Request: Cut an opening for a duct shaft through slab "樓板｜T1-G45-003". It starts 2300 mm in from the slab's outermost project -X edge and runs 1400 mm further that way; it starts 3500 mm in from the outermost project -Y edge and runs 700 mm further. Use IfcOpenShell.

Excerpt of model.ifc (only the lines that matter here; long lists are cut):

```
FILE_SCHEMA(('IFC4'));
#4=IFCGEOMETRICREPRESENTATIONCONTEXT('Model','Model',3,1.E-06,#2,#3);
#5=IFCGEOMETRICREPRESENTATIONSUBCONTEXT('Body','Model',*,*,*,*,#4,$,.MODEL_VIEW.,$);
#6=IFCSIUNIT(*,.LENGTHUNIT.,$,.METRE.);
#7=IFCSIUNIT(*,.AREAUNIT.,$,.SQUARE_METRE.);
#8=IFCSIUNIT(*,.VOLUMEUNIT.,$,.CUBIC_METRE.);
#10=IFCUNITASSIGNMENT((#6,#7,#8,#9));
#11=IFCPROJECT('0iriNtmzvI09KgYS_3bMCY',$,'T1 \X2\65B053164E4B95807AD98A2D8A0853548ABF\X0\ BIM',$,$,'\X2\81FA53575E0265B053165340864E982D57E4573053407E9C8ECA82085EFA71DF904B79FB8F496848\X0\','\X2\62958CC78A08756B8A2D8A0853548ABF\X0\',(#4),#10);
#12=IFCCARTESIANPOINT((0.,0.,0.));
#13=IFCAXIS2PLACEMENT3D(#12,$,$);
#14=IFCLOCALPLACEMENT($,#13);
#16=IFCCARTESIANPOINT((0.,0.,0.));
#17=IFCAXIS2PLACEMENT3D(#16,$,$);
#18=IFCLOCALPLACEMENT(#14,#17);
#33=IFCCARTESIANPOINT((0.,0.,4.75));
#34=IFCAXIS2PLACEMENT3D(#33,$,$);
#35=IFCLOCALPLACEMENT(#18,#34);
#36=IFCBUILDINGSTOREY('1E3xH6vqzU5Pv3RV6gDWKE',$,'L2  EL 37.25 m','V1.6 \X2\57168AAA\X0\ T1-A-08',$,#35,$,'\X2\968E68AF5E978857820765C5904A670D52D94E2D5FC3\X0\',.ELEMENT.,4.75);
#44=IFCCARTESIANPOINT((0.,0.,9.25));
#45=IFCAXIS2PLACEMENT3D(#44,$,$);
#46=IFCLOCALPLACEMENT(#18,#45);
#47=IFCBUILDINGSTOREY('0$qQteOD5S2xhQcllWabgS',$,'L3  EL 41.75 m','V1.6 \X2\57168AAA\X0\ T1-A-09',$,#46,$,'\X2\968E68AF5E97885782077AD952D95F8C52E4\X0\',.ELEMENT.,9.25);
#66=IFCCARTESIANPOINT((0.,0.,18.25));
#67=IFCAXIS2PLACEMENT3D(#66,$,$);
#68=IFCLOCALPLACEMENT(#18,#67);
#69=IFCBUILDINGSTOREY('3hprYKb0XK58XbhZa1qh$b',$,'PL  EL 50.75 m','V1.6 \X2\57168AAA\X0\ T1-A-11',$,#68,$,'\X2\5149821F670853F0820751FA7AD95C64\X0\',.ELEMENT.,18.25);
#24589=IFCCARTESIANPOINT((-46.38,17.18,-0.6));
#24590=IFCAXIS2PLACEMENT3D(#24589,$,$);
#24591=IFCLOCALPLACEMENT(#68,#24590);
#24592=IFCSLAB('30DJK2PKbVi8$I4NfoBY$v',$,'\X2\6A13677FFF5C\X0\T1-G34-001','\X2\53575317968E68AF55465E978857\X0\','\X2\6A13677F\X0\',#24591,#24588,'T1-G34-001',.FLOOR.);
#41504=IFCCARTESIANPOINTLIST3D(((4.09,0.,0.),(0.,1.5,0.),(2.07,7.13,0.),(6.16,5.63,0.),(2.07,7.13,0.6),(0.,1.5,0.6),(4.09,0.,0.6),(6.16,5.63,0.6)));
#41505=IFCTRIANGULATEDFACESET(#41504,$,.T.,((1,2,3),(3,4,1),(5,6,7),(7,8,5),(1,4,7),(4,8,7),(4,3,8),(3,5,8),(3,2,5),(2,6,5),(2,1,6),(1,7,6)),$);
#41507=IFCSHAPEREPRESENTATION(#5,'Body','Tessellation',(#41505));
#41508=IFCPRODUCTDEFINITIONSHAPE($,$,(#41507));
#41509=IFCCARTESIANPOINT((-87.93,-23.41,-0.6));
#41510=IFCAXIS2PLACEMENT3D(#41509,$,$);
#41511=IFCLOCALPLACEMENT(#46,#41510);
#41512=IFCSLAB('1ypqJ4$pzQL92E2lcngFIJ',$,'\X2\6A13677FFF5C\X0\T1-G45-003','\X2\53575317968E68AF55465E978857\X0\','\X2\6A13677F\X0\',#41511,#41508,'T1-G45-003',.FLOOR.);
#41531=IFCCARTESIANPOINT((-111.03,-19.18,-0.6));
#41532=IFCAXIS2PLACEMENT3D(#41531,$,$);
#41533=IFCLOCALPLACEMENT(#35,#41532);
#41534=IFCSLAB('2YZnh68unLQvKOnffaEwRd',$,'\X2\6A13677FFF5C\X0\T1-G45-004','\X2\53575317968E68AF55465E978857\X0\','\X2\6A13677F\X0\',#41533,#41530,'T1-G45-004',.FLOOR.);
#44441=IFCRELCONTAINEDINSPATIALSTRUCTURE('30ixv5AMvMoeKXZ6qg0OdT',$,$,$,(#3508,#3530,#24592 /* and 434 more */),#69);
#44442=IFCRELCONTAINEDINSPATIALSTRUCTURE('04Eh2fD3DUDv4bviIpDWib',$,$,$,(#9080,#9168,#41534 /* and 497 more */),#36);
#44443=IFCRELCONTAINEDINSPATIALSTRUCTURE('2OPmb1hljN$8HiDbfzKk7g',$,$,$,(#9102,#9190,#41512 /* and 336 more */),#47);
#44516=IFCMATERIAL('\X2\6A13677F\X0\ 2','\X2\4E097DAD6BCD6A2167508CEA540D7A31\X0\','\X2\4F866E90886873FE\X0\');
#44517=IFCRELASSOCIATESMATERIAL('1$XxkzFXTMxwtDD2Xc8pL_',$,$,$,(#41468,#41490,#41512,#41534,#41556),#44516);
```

```python
import numpy as np
import ifcopenshell
import ifcopenshell.api.feature
import ifcopenshell.api.geometry
import ifcopenshell.api.root
import ifcopenshell.geom
import ifcopenshell.util.placement
import ifcopenshell.util.representation
import ifcopenshell.util.shape
import ifcopenshell.util.unit

model = ifcopenshell.open("model.ifc")
unit_scale = ifcopenshell.util.unit.calculate_unit_scale(model)
settings = ifcopenshell.geom.settings()


def volume(element):
    """Net volume in cubic metres, openings subtracted."""
    shape = ifcopenshell.geom.create_shape(settings, element)
    return ifcopenshell.util.shape.get_volume(shape.geometry)


slab = model.by_guid("1ypqJ4$pzQL92E2lcngFIJ")
before = volume(slab)

# Extent in the slab's own axes, in metres. The edges named are its -X and -Y sides.
slab_shape = ifcopenshell.geom.create_shape(settings, slab)
vertices = ifcopenshell.util.shape.get_vertices(slab_shape.geometry)
x_min, y_min, bottom = vertices.min(axis=0)
top = vertices[:, 2].max()

opening = ifcopenshell.api.root.create_entity(model, ifc_class="IfcOpeningElement", name="Duct shaft opening", predefined_type="OPENING")
context = ifcopenshell.util.representation.get_context(model, "Model", "Body", "MODEL_VIEW")
width, depth = 1.4, 0.7
outline = [(0.0, 0.0), (width, 0.0), (width, depth), (0.0, depth), (0.0, 0.0)]
# Overshoot both faces by 50 mm so the cut is clean.
shape = ifcopenshell.api.geometry.add_slab_representation(
    model, context=context, depth=top - bottom + 0.1, polyline=outline
)
ifcopenshell.api.geometry.assign_representation(model, product=opening, representation=shape)

matrix = ifcopenshell.util.placement.get_local_placement(slab.ObjectPlacement)
matrix[:, 3] = matrix @ np.append(np.array([x_min + 2.3, y_min + 3.5, bottom - 0.05]) / unit_scale, 1.0)
ifcopenshell.api.geometry.edit_object_placement(model, product=opening, matrix=matrix, is_si=False)
ifcopenshell.api.feature.add_feature(model, feature=opening, element=slab)

after = volume(slab)

print(f"slab volume {before:.3f} -> {after:.3f} m3")

model.write("model-out.ifc")
```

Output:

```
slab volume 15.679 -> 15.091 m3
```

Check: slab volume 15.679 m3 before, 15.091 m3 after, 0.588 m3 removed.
